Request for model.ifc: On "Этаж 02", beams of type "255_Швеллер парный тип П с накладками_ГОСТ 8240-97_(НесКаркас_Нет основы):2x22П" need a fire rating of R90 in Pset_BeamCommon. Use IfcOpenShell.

First a look at what the model holds.

```python
import ifcopenshell
import ifcopenshell.util.element

model = ifcopenshell.open("model.ifc")
print(model.schema)
storey = next(s for s in model.by_type("IfcBuildingStorey") if s.Name == "Этаж 02")
beams = [e for e in ifcopenshell.util.element.get_decomposition(storey) if e.is_a("IfcBeam")]
seen = {}
for e in beams:
    element_type = ifcopenshell.util.element.get_type(e)
    key = (element_type.Name if element_type != e and element_type else None, ifcopenshell.util.element.get_pset(e, "Pset_BeamCommon", "FireRating"))
    seen[key] = seen.get(key, 0) + 1
for (name, value), count in sorted(seen.items(), key=str):
    print(count, "x", name, "|", value)
```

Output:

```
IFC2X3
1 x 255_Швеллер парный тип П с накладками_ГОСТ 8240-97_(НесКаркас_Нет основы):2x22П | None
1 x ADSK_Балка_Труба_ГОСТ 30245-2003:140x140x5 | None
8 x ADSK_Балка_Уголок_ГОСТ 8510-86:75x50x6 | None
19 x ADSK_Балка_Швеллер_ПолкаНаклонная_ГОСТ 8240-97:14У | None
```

```python
import ifcopenshell
import ifcopenshell.api.pset
import ifcopenshell.util.element

model = ifcopenshell.open("model.ifc")

storey = next(s for s in model.by_type("IfcBuildingStorey") if s.Name == "Этаж 02")
beams = [e for e in ifcopenshell.util.element.get_decomposition(storey) if e.is_a("IfcBeam")]

count = 0
for e in beams:
    element_type = ifcopenshell.util.element.get_type(e)
    if element_type in (None, e) or element_type.Name != "255_Швеллер парный тип П с накладками_ГОСТ 8240-97_(НесКаркас_Нет основы):2x22П":
        continue
    # add_pset returns the element's existing set when there is one.
    pset = ifcopenshell.api.pset.add_pset(model, product=e, name="Pset_BeamCommon")
    ifcopenshell.api.pset.edit_pset(model, pset=pset, properties={"FireRating": "R90"})
    count += 1

print(count, "beams updated")

model.write("model_rev.ifc")
```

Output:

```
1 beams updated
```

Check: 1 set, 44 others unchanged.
